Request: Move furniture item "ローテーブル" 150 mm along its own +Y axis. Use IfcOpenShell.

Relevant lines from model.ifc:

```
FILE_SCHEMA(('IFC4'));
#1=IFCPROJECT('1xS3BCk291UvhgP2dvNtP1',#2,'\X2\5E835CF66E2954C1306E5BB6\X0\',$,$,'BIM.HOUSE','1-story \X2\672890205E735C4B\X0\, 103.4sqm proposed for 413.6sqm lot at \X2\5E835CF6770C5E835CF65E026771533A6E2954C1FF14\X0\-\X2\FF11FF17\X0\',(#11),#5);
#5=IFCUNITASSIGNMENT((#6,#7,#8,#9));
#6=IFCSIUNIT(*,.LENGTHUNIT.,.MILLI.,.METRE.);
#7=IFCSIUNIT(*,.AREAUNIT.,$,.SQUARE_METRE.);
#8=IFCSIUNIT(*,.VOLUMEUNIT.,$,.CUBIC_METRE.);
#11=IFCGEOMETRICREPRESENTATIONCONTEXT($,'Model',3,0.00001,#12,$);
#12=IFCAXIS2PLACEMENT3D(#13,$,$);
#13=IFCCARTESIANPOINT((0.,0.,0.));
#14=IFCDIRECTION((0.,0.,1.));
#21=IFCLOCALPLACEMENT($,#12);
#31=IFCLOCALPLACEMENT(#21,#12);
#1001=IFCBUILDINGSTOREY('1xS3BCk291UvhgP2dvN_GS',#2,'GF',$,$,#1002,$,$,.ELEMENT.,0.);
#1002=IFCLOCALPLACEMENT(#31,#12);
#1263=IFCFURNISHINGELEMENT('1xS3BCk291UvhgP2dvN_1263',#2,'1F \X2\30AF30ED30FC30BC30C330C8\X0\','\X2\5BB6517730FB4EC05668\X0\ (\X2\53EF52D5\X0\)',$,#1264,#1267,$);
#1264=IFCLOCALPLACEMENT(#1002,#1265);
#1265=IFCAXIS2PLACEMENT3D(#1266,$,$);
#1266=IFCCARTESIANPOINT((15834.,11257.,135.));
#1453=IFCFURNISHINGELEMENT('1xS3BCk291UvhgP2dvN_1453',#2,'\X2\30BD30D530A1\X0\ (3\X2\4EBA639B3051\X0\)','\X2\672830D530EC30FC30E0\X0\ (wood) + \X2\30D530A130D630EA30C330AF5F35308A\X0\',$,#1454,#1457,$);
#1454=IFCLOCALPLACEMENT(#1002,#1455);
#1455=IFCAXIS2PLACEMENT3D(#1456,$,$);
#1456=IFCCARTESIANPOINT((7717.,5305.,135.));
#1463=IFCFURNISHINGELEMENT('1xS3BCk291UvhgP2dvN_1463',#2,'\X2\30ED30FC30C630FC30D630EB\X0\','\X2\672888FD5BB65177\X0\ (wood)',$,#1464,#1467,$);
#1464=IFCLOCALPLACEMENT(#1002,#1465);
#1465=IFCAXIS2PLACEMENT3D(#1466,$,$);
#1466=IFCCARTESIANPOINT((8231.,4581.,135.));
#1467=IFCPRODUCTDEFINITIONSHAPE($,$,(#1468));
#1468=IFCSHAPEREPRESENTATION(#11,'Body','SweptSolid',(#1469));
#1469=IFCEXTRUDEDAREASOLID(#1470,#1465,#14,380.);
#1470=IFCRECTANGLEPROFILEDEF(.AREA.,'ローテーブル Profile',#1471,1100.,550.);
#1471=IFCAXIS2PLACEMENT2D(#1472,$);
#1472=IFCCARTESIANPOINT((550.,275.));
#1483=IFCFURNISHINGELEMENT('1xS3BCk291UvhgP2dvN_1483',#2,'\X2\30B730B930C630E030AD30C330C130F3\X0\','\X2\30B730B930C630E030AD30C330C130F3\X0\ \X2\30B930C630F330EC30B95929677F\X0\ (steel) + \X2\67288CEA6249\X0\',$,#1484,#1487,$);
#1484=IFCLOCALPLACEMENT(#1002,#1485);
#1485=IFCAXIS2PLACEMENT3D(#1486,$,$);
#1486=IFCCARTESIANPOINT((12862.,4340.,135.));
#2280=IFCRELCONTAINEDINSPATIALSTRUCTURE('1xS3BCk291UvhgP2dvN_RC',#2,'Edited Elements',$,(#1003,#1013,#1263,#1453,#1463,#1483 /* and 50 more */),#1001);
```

```python
import ifcopenshell
import ifcopenshell.api.geometry
import ifcopenshell.util.placement

model = ifcopenshell.open("model.ifc")

item = model.by_id(1463)
matrix = ifcopenshell.util.placement.get_local_placement(item.ObjectPlacement)
matrix[:3, 3] += matrix[:3, 1] * 150.0
ifcopenshell.api.geometry.edit_object_placement(model, product=item, matrix=matrix, is_si=False)

print(ifcopenshell.util.placement.get_local_placement(item.ObjectPlacement).round(3) + 0.0)

model.write("model_v2.ifc")
```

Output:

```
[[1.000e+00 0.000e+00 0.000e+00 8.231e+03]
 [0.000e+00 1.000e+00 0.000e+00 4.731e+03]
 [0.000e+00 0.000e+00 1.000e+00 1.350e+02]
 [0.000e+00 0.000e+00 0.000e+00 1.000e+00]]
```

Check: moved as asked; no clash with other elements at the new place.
